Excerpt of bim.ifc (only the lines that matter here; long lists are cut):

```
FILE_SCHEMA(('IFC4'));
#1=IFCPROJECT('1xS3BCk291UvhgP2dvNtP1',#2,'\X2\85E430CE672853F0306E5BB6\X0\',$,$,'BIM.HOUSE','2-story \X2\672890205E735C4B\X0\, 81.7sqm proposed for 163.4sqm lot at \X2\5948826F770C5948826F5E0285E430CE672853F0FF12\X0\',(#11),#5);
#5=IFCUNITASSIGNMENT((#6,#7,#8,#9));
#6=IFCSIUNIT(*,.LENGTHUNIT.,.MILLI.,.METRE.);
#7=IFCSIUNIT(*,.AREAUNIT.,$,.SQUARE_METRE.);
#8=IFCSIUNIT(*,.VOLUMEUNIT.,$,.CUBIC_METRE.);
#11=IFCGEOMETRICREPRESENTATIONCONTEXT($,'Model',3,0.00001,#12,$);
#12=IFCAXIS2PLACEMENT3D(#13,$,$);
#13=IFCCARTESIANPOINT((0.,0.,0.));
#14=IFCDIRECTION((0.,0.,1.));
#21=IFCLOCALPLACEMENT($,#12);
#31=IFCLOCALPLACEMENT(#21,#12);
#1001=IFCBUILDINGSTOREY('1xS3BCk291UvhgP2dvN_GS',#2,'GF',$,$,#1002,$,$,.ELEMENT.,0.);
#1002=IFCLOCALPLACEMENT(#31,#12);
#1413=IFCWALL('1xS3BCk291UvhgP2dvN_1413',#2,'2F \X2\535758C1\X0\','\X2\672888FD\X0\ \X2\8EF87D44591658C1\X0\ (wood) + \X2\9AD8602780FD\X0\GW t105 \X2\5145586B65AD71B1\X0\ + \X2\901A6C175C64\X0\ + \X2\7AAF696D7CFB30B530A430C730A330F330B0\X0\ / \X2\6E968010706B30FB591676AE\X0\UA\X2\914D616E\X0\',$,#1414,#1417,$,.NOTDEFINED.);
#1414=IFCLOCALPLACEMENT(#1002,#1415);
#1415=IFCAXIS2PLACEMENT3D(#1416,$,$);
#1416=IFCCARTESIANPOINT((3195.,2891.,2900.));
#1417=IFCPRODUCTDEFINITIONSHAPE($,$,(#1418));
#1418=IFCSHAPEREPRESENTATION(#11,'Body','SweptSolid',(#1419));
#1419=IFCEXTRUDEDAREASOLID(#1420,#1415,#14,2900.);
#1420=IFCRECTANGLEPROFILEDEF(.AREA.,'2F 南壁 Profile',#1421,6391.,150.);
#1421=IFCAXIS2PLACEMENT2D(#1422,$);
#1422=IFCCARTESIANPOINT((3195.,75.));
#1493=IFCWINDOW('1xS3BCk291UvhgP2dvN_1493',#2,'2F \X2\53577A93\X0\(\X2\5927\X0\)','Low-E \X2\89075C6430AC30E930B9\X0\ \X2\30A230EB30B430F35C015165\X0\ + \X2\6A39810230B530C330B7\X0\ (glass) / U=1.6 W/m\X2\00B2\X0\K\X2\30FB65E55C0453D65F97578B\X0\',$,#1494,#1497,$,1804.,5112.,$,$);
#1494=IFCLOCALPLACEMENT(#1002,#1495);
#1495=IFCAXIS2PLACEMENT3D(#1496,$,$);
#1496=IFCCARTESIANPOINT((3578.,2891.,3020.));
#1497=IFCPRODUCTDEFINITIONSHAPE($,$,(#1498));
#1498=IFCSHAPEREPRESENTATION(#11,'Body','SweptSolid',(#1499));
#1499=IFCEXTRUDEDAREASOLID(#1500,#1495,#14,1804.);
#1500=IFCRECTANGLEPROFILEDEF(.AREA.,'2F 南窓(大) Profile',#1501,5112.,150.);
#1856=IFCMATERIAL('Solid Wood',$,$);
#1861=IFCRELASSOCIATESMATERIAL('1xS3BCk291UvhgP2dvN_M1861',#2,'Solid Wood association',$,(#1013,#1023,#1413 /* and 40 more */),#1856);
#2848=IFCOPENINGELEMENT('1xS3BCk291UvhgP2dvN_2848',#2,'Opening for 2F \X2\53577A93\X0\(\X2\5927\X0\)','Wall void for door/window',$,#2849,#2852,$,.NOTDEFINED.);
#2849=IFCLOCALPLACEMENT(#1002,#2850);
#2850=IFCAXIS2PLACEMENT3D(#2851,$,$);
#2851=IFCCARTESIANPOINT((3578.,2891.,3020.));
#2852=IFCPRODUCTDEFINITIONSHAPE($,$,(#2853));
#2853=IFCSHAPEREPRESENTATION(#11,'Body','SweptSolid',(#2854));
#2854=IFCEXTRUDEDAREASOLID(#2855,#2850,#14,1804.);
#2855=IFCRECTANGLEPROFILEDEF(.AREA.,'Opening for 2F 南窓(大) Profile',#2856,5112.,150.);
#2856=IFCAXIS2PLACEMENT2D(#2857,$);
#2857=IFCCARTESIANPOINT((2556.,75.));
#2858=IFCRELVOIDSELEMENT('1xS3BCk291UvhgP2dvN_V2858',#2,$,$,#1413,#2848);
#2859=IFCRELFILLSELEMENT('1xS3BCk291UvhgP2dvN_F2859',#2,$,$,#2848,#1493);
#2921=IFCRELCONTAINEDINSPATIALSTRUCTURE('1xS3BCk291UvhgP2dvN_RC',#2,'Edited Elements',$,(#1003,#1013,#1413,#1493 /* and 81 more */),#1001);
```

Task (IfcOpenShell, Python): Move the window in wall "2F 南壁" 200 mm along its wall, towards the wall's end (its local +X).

```python
import ifcopenshell
import ifcopenshell.api.geometry
import ifcopenshell.util.placement

model = ifcopenshell.open("bim.ifc")

window = model.by_id(1493)
opening = window.FillsVoids[0].RelatingOpeningElement
wall = opening.VoidsElements[0].RelatingBuildingElement

wall_matrix = ifcopenshell.util.placement.get_local_placement(wall.ObjectPlacement)
shift = wall_matrix[:3, 0] * 200.0
before = ifcopenshell.util.placement.get_local_placement(window.ObjectPlacement)[:3, 3].copy()

# The window is not placed relative to its opening, so move both.
for product in (opening, window):
    matrix = ifcopenshell.util.placement.get_local_placement(product.ObjectPlacement)
    matrix[:3, 3] += shift
    ifcopenshell.api.geometry.edit_object_placement(model, product=product, matrix=matrix, is_si=False)

after = ifcopenshell.util.placement.get_local_placement(window.ObjectPlacement)[:3, 3]
print("window moved by", (after - before).round(3) + 0.0)

model.write("bim-out.ifc")
```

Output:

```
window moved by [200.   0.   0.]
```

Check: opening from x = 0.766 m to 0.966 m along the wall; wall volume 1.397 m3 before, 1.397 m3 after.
